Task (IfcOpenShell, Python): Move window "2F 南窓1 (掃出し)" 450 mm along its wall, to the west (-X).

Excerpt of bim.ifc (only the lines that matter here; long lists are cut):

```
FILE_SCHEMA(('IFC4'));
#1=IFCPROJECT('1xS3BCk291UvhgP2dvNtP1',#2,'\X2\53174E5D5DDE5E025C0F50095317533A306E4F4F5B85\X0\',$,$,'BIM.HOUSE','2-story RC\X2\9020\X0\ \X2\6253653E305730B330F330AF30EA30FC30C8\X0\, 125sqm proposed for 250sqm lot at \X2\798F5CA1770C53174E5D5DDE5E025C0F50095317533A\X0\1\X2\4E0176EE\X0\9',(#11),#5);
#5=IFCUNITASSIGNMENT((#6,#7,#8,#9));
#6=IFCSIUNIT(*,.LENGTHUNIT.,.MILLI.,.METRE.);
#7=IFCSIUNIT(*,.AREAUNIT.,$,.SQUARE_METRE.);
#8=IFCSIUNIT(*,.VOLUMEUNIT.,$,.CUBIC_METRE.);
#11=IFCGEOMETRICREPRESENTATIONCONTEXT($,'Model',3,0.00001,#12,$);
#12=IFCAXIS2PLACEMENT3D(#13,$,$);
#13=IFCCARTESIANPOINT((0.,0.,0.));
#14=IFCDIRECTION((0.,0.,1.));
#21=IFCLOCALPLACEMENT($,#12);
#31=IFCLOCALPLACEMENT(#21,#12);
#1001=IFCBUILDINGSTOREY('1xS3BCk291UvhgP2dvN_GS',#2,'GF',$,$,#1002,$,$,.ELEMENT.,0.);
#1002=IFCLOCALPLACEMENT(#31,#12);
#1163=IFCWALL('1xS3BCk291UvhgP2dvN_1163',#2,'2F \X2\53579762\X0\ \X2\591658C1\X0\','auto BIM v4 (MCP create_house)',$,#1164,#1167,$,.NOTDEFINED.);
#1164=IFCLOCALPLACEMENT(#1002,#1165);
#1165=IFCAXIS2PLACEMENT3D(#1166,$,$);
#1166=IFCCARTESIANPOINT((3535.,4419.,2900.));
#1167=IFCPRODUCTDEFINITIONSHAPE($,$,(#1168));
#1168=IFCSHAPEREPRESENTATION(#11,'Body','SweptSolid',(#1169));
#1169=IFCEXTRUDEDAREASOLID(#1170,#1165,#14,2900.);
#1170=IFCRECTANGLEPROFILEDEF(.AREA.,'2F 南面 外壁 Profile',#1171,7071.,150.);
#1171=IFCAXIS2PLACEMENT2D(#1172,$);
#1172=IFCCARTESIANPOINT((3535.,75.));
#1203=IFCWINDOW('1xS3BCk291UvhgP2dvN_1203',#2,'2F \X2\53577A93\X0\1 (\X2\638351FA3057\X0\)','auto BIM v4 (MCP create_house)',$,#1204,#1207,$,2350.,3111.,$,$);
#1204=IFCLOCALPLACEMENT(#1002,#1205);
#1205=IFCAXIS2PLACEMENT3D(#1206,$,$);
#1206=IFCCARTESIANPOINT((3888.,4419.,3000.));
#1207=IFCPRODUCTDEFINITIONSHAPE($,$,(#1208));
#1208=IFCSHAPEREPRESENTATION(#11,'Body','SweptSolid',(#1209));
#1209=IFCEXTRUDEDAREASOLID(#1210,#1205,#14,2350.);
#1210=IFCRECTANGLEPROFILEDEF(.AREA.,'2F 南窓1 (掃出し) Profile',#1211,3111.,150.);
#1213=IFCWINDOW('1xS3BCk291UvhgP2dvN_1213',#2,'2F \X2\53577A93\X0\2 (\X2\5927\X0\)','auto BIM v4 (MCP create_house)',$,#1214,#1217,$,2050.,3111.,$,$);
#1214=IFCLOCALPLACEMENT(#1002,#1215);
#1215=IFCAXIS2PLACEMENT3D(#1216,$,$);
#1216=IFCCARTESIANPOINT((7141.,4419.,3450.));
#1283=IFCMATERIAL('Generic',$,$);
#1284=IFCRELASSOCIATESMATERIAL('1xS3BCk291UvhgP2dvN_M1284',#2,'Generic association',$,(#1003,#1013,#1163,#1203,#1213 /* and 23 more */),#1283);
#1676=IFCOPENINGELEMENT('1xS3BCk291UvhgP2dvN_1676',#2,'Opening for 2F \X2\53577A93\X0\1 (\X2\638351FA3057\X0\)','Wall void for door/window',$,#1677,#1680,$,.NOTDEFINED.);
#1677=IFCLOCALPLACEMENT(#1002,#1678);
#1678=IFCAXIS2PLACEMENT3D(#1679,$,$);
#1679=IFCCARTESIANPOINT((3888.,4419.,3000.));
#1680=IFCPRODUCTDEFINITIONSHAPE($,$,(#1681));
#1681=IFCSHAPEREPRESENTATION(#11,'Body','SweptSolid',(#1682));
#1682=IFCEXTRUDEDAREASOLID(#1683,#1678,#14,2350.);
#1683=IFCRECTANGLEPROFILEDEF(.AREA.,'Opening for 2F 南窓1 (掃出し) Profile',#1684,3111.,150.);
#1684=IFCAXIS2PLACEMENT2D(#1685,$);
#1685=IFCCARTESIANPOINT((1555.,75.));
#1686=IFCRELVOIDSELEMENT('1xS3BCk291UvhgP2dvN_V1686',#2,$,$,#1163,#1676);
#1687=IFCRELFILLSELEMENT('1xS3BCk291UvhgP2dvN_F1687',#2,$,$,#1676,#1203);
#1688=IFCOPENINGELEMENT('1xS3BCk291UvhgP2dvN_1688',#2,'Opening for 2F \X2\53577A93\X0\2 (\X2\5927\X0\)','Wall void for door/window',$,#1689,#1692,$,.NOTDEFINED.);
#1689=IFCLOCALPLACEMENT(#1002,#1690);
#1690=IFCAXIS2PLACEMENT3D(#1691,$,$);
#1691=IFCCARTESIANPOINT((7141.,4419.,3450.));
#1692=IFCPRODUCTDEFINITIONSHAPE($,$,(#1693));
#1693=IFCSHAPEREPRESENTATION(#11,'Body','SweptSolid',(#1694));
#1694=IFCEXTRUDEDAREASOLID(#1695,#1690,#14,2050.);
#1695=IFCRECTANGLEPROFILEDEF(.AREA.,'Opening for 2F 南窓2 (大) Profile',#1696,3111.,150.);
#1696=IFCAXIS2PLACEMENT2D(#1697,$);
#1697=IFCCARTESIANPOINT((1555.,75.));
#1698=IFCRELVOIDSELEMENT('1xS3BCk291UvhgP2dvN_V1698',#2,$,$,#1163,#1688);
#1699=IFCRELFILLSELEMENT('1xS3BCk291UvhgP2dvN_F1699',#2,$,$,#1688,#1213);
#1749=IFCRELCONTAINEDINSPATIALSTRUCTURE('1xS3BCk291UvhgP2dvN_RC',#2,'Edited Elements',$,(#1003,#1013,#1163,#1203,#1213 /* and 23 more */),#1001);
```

```python
import ifcopenshell
import ifcopenshell.api.geometry
import ifcopenshell.util.placement
import ifcopenshell.util.unit

model = ifcopenshell.open("bim.ifc")
unit_scale = ifcopenshell.util.unit.calculate_unit_scale(model)

window = model.by_id(1203)
opening = window.FillsVoids[0].RelatingOpeningElement
wall = opening.VoidsElements[0].RelatingBuildingElement

wall_matrix = ifcopenshell.util.placement.get_local_placement(wall.ObjectPlacement)
shift = wall_matrix[:3, 0] * -0.45 / unit_scale
before = ifcopenshell.util.placement.get_local_placement(window.ObjectPlacement)[:3, 3].copy()

# The window is not placed relative to its opening, so move both.
for product in (opening, window):
    matrix = ifcopenshell.util.placement.get_local_placement(product.ObjectPlacement)
    matrix[:3, 3] += shift
    ifcopenshell.api.geometry.edit_object_placement(model, product=product, matrix=matrix, is_si=False)

after = ifcopenshell.util.placement.get_local_placement(window.ObjectPlacement)[:3, 3]
print("window moved by", (after - before).round(3) + 0.0)

model.write("bim-out.ifc")
```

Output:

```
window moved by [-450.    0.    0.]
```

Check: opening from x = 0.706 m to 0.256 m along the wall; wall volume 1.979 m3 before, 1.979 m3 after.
